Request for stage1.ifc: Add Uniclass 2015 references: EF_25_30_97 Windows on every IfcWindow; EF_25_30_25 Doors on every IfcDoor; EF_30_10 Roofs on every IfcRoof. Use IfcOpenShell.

First a look at what the model holds.

```python
import ifcopenshell

model = ifcopenshell.open("stage1.ifc")
print(model.schema)
print("classifications:", [c.Name for c in model.by_type("IfcClassification")])
for ifc_class in ("IfcDoor", "IfcRoof", "IfcStair", "IfcWall", "IfcWindow"):
    print(ifc_class, len(model.by_type(ifc_class)))
```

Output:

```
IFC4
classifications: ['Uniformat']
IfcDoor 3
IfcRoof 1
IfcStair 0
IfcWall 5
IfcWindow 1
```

```python
import ifcopenshell
import ifcopenshell.api.classification

model = ifcopenshell.open("stage1.ifc")

system = ifcopenshell.api.classification.add_classification(model, classification="Uniclass 2015")

codes = {
    "IfcWindow": ("EF_25_30_97", "Windows"),
    "IfcDoor": ("EF_25_30_25", "Doors"),
    "IfcRoof": ("EF_30_10", "Roofs"),
}
for ifc_class, (code, name) in codes.items():
    products = model.by_type(ifc_class)
    ifcopenshell.api.classification.add_reference(
        model, products=products, classification=system, identification=code, name=name
    )
    print(code, len(products))

model.write("stage1_edited.ifc")
```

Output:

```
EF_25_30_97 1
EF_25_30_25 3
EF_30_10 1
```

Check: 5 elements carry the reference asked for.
